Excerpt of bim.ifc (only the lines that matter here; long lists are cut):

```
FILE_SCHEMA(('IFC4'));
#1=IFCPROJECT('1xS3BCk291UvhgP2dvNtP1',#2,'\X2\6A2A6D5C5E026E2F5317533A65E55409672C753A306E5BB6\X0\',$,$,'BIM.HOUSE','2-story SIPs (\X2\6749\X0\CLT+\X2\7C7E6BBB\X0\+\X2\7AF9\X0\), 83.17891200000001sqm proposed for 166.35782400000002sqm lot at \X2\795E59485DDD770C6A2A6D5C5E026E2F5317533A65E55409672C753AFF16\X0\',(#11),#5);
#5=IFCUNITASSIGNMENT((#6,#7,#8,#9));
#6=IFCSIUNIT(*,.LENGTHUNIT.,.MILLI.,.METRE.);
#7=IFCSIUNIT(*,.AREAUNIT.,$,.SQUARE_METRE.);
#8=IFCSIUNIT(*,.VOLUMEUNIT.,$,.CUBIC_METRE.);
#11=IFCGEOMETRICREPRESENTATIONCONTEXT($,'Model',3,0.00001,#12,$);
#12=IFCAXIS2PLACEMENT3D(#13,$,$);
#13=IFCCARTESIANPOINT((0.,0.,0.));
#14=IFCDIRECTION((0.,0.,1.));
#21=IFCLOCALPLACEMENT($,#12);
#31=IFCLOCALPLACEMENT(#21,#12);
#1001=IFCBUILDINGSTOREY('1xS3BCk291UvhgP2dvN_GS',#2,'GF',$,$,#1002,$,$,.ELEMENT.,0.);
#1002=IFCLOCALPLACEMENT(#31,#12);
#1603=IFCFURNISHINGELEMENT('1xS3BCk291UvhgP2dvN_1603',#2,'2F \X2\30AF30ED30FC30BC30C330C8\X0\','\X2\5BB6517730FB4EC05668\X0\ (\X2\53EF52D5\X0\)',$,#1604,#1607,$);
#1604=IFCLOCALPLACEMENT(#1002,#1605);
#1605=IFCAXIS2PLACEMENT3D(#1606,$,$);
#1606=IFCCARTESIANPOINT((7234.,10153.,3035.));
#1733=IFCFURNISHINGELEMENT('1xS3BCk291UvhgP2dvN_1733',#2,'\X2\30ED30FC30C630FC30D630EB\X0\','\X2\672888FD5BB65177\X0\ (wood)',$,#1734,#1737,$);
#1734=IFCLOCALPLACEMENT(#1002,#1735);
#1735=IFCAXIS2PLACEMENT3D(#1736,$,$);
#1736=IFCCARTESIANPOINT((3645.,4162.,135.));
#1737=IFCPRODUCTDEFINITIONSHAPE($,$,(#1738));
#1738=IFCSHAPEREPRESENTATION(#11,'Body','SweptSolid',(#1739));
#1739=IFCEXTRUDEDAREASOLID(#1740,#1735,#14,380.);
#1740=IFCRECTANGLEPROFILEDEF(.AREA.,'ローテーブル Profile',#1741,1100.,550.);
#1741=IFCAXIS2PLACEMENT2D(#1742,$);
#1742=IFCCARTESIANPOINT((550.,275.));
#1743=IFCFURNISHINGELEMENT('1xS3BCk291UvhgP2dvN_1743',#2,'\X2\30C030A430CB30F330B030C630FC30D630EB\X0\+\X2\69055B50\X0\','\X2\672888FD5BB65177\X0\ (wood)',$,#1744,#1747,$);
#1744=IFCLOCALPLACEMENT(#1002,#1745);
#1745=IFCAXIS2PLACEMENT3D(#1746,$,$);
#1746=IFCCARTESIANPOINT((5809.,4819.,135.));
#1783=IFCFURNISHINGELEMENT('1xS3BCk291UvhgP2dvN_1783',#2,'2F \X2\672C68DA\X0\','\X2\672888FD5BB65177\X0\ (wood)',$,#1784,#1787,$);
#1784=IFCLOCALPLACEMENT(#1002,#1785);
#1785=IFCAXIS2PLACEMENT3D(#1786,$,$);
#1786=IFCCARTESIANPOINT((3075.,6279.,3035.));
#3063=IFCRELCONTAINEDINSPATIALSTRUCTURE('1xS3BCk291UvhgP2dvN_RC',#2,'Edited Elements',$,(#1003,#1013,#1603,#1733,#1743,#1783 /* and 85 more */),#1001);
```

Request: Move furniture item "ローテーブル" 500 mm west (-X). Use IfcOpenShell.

```python
import ifcopenshell
import ifcopenshell.api.geometry
import ifcopenshell.util.placement
import ifcopenshell.util.unit

model = ifcopenshell.open("bim.ifc")
unit_scale = ifcopenshell.util.unit.calculate_unit_scale(model)

item = model.by_guid("1xS3BCk291UvhgP2dvN_1733")
matrix = ifcopenshell.util.placement.get_local_placement(item.ObjectPlacement)
matrix[0, 3] -= 0.5 / unit_scale
ifcopenshell.api.geometry.edit_object_placement(model, product=item, matrix=matrix, is_si=False)

print(ifcopenshell.util.placement.get_local_placement(item.ObjectPlacement).round(3) + 0.0)

model.write("bim_edited.ifc")
```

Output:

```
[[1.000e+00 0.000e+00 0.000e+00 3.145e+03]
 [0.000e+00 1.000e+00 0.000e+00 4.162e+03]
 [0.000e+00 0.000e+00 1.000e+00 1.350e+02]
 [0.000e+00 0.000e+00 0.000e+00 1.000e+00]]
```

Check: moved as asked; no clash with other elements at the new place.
